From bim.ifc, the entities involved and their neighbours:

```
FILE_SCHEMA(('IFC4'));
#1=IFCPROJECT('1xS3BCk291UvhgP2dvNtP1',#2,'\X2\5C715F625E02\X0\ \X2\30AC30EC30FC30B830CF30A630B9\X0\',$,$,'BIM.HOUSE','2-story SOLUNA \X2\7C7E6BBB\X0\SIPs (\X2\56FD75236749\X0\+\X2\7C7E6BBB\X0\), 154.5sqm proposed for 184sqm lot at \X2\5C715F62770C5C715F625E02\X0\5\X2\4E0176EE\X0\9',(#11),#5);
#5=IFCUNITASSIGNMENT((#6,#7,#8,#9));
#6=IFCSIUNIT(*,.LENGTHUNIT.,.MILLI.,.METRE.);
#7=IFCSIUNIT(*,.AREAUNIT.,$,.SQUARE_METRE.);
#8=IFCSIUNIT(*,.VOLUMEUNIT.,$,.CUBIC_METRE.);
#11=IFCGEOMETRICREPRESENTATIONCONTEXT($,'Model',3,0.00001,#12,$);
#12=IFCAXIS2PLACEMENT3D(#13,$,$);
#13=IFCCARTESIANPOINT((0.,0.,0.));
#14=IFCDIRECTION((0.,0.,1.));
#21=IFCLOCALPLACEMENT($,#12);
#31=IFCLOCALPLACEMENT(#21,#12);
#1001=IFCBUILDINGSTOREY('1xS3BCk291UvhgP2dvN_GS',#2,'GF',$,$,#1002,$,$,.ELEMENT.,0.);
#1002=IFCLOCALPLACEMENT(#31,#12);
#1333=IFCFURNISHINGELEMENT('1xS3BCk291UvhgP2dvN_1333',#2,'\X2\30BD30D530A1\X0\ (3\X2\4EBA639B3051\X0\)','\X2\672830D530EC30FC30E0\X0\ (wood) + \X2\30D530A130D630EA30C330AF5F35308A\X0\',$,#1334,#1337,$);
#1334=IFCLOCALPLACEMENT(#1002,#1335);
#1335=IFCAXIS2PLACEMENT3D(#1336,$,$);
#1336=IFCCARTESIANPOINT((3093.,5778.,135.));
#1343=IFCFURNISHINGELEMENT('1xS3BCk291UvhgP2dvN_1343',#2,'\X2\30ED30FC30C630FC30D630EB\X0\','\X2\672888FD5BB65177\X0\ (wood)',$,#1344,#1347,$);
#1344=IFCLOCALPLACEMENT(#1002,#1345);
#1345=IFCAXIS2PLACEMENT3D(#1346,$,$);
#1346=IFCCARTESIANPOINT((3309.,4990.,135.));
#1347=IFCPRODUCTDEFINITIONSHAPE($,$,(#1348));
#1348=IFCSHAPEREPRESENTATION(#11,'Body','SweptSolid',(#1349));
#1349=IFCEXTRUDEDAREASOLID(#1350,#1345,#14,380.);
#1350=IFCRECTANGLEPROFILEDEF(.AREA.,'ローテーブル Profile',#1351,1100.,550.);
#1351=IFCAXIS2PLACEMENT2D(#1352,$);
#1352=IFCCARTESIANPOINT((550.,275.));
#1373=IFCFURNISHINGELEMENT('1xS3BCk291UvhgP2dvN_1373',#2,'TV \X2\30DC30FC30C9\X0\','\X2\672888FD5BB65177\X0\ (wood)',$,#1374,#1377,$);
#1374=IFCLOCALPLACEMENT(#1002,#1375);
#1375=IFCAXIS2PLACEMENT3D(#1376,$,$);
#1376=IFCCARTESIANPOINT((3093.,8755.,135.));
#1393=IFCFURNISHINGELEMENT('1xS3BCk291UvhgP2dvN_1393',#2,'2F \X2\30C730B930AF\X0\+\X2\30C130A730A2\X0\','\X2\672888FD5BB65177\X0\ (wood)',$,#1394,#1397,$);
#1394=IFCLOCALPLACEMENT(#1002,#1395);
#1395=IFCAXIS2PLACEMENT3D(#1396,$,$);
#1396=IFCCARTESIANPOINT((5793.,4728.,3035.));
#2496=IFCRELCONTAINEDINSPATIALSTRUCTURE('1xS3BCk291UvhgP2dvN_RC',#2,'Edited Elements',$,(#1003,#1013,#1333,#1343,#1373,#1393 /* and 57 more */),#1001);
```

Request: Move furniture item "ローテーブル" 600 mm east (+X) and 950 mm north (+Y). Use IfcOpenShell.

```python
import ifcopenshell
import ifcopenshell.api.geometry
import ifcopenshell.util.placement
import ifcopenshell.util.unit

model = ifcopenshell.open("bim.ifc")
unit_scale = ifcopenshell.util.unit.calculate_unit_scale(model)

item = model.by_guid("1xS3BCk291UvhgP2dvN_1343")
matrix = ifcopenshell.util.placement.get_local_placement(item.ObjectPlacement)
matrix[0, 3] += 0.6 / unit_scale
matrix[1, 3] += 0.95 / unit_scale
ifcopenshell.api.geometry.edit_object_placement(model, product=item, matrix=matrix, is_si=False)

print(ifcopenshell.util.placement.get_local_placement(item.ObjectPlacement).round(3) + 0.0)

model.write("bim_edited.ifc")
```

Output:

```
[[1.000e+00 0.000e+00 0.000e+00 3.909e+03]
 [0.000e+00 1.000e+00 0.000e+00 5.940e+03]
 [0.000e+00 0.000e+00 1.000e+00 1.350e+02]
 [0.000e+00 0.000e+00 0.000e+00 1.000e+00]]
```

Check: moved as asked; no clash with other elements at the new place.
